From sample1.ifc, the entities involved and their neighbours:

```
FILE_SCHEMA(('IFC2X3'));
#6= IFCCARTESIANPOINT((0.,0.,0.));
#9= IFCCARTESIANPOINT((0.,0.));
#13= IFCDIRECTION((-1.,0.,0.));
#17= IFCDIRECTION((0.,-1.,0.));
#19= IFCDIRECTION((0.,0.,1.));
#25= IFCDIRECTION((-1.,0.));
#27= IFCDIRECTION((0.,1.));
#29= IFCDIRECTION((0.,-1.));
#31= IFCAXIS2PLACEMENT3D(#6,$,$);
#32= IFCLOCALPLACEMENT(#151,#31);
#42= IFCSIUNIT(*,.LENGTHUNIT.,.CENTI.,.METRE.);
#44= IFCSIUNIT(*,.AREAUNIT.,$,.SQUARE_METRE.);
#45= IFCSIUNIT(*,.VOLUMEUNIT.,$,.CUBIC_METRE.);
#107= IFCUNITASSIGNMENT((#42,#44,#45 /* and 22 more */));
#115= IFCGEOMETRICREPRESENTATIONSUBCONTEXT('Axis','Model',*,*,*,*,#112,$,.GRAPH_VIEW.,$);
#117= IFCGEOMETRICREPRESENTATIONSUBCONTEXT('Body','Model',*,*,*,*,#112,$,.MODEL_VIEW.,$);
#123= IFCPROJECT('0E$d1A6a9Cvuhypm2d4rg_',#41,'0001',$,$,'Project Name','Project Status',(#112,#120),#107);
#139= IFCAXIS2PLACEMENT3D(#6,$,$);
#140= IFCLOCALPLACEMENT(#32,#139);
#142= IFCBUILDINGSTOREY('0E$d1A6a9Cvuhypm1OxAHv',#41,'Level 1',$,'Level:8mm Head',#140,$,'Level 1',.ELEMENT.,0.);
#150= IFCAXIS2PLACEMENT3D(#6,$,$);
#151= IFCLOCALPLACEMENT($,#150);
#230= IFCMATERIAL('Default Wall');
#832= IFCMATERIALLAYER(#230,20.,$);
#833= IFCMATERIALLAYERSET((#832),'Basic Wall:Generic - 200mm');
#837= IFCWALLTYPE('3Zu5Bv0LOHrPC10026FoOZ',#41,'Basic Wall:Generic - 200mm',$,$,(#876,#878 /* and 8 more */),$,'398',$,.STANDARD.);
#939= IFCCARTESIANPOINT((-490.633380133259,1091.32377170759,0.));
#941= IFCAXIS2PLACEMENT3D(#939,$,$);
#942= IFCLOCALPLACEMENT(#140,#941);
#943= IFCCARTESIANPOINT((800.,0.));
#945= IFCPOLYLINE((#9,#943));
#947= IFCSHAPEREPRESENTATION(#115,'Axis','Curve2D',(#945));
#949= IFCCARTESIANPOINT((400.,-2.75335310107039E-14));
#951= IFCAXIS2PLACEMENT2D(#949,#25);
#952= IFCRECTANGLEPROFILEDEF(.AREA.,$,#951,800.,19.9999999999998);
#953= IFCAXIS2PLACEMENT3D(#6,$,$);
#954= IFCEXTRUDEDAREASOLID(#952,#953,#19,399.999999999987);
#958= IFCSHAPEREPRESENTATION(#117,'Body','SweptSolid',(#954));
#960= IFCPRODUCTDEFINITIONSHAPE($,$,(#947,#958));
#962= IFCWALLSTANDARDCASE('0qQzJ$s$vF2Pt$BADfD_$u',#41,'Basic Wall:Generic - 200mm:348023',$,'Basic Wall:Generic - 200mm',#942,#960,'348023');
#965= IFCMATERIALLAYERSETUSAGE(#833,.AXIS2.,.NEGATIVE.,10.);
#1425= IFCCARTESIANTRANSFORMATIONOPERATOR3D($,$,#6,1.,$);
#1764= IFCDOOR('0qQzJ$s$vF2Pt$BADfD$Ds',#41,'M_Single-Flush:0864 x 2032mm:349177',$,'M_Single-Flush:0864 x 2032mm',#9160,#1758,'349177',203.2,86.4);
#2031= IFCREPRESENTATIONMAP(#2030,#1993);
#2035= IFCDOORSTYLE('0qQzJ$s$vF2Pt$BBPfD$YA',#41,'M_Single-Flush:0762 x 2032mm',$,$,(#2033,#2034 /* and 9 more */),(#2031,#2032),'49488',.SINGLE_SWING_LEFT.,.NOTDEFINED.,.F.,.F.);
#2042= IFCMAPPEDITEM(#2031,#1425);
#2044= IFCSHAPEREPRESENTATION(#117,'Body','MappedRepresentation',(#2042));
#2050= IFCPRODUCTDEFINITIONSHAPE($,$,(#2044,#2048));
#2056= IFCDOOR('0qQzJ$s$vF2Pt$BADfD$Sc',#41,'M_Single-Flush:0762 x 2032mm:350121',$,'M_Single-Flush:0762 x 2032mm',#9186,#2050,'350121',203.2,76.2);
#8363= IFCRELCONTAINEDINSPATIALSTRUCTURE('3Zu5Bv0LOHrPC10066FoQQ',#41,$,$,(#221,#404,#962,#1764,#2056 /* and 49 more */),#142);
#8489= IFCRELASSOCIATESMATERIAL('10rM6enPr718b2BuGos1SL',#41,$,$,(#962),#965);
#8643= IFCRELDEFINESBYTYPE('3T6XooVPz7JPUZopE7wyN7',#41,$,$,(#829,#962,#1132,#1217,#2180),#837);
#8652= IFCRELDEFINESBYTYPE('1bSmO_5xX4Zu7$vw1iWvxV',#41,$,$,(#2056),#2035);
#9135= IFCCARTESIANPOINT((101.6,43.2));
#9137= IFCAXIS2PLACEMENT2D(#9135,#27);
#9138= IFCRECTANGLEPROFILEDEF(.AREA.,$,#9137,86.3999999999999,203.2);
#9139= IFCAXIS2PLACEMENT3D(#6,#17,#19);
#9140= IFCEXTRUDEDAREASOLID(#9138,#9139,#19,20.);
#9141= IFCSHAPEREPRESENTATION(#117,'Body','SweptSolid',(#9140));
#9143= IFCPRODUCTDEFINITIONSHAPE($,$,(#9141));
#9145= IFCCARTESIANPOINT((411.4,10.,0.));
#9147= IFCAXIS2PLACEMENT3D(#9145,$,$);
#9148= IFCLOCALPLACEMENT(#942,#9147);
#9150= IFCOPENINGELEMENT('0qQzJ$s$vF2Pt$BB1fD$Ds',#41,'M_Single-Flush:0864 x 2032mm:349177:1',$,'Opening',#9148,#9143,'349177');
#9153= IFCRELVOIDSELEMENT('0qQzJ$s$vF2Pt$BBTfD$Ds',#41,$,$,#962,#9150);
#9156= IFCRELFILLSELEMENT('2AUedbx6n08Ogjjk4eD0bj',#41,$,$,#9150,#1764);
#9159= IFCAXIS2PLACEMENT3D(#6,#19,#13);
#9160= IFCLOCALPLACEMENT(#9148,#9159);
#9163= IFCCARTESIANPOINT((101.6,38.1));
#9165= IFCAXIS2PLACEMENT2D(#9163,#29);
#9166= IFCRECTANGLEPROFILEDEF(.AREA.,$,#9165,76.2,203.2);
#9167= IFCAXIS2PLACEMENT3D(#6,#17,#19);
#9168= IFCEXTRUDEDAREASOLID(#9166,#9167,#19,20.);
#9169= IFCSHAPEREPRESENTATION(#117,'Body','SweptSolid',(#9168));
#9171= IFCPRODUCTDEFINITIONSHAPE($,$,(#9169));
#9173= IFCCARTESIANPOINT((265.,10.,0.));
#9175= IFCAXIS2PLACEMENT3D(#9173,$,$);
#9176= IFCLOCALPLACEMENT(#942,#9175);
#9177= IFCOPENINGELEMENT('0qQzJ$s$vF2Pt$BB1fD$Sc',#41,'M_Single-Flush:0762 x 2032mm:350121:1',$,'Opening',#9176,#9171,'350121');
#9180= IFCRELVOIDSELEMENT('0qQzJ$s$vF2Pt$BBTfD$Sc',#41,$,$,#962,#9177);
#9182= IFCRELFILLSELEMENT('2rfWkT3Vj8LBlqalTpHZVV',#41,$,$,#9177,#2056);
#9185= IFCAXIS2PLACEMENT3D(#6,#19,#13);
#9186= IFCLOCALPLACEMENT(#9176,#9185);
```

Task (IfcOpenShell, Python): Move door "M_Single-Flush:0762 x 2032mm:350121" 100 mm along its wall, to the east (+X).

```python
import ifcopenshell
import ifcopenshell.api.geometry
import ifcopenshell.util.placement
import ifcopenshell.util.unit

model = ifcopenshell.open("sample1.ifc")
unit_scale = ifcopenshell.util.unit.calculate_unit_scale(model)

door = model.by_guid("0qQzJ$s$vF2Pt$BADfD$Sc")
opening = door.FillsVoids[0].RelatingOpeningElement
wall = opening.VoidsElements[0].RelatingBuildingElement

wall_matrix = ifcopenshell.util.placement.get_local_placement(wall.ObjectPlacement)
shift = wall_matrix[:3, 0] * 0.1 / unit_scale
before = ifcopenshell.util.placement.get_local_placement(door.ObjectPlacement)[:3, 3].copy()

# The door is placed relative to its opening, so it follows when the opening moves.
matrix = ifcopenshell.util.placement.get_local_placement(opening.ObjectPlacement)
matrix[:3, 3] += shift
ifcopenshell.api.geometry.edit_object_placement(
    model, product=opening, matrix=matrix, is_si=False, should_transform_children=True
)

after = ifcopenshell.util.placement.get_local_placement(door.ObjectPlacement)[:3, 3]
print("door moved by", (after - before).round(3) + 0.0)

model.write("sample1_v2.ifc")
```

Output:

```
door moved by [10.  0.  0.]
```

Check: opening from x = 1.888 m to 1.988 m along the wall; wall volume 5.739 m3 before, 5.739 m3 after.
